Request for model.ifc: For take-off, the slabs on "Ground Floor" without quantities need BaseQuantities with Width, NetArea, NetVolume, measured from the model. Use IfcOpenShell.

First a look at what the model holds.

```python
import ifcopenshell
import ifcopenshell.util.element
import ifcopenshell.util.unit

model = ifcopenshell.open("model.ifc")
print(model.schema)
for unit_type in ("LENGTHUNIT", "AREAUNIT", "VOLUMEUNIT"):
    print(unit_type, ifcopenshell.util.unit.calculate_unit_scale(model, unit_type))
storey = next(s for s in model.by_type("IfcBuildingStorey") if s.Name == "Ground Floor")
slabs = [e for e in ifcopenshell.util.element.get_decomposition(storey) if e.is_a("IfcSlab")]
for e in sorted(slabs, key=lambda e: e.id()):
    print(e.id(), e.is_a(), e.Name, list(ifcopenshell.util.element.get_psets(e, qtos_only=True)), sep=" | ")
```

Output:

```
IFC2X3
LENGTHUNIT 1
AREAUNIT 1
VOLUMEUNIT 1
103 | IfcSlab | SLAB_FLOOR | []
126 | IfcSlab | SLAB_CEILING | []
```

```python
import ifcopenshell
import ifcopenshell.api.pset
import ifcopenshell.geom
import ifcopenshell.util.element
import ifcopenshell.util.shape
import ifcopenshell.util.unit

model = ifcopenshell.open("model.ifc")
unit_scale = ifcopenshell.util.unit.calculate_unit_scale(model)
area_scale = ifcopenshell.util.unit.calculate_unit_scale(model, "AREAUNIT")
volume_scale = ifcopenshell.util.unit.calculate_unit_scale(model, "VOLUMEUNIT")
settings = ifcopenshell.geom.settings()

storey = next(s for s in model.by_type("IfcBuildingStorey") if s.Name == "Ground Floor")
slabs = [e for e in ifcopenshell.util.element.get_decomposition(storey) if e.is_a("IfcSlab")]

for e in sorted(slabs, key=lambda e: e.id()):
    if ifcopenshell.util.element.get_psets(e, qtos_only=True, should_inherit=False):
        continue
    # Geometry comes back in metres, in the element's own axes.
    shape = ifcopenshell.geom.create_shape(settings, e)
    values = {
        "Width": ifcopenshell.util.shape.get_z(shape.geometry) / unit_scale,
        "NetArea": ifcopenshell.util.shape.get_footprint_area(shape.geometry) / area_scale,
        "NetVolume": ifcopenshell.util.shape.get_volume(shape.geometry) / volume_scale,
    }
    qto = ifcopenshell.api.pset.add_qto(model, product=e, name="BaseQuantities")
    ifcopenshell.api.pset.edit_qto(model, qto=qto, properties=values)
    print(e.id(), {k: round(v, 3) for k, v in values.items()})

model.write("model_rev.ifc")
```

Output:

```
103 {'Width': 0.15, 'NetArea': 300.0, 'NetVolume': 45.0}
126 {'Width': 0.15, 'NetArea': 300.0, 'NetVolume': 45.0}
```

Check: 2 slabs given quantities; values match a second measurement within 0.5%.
